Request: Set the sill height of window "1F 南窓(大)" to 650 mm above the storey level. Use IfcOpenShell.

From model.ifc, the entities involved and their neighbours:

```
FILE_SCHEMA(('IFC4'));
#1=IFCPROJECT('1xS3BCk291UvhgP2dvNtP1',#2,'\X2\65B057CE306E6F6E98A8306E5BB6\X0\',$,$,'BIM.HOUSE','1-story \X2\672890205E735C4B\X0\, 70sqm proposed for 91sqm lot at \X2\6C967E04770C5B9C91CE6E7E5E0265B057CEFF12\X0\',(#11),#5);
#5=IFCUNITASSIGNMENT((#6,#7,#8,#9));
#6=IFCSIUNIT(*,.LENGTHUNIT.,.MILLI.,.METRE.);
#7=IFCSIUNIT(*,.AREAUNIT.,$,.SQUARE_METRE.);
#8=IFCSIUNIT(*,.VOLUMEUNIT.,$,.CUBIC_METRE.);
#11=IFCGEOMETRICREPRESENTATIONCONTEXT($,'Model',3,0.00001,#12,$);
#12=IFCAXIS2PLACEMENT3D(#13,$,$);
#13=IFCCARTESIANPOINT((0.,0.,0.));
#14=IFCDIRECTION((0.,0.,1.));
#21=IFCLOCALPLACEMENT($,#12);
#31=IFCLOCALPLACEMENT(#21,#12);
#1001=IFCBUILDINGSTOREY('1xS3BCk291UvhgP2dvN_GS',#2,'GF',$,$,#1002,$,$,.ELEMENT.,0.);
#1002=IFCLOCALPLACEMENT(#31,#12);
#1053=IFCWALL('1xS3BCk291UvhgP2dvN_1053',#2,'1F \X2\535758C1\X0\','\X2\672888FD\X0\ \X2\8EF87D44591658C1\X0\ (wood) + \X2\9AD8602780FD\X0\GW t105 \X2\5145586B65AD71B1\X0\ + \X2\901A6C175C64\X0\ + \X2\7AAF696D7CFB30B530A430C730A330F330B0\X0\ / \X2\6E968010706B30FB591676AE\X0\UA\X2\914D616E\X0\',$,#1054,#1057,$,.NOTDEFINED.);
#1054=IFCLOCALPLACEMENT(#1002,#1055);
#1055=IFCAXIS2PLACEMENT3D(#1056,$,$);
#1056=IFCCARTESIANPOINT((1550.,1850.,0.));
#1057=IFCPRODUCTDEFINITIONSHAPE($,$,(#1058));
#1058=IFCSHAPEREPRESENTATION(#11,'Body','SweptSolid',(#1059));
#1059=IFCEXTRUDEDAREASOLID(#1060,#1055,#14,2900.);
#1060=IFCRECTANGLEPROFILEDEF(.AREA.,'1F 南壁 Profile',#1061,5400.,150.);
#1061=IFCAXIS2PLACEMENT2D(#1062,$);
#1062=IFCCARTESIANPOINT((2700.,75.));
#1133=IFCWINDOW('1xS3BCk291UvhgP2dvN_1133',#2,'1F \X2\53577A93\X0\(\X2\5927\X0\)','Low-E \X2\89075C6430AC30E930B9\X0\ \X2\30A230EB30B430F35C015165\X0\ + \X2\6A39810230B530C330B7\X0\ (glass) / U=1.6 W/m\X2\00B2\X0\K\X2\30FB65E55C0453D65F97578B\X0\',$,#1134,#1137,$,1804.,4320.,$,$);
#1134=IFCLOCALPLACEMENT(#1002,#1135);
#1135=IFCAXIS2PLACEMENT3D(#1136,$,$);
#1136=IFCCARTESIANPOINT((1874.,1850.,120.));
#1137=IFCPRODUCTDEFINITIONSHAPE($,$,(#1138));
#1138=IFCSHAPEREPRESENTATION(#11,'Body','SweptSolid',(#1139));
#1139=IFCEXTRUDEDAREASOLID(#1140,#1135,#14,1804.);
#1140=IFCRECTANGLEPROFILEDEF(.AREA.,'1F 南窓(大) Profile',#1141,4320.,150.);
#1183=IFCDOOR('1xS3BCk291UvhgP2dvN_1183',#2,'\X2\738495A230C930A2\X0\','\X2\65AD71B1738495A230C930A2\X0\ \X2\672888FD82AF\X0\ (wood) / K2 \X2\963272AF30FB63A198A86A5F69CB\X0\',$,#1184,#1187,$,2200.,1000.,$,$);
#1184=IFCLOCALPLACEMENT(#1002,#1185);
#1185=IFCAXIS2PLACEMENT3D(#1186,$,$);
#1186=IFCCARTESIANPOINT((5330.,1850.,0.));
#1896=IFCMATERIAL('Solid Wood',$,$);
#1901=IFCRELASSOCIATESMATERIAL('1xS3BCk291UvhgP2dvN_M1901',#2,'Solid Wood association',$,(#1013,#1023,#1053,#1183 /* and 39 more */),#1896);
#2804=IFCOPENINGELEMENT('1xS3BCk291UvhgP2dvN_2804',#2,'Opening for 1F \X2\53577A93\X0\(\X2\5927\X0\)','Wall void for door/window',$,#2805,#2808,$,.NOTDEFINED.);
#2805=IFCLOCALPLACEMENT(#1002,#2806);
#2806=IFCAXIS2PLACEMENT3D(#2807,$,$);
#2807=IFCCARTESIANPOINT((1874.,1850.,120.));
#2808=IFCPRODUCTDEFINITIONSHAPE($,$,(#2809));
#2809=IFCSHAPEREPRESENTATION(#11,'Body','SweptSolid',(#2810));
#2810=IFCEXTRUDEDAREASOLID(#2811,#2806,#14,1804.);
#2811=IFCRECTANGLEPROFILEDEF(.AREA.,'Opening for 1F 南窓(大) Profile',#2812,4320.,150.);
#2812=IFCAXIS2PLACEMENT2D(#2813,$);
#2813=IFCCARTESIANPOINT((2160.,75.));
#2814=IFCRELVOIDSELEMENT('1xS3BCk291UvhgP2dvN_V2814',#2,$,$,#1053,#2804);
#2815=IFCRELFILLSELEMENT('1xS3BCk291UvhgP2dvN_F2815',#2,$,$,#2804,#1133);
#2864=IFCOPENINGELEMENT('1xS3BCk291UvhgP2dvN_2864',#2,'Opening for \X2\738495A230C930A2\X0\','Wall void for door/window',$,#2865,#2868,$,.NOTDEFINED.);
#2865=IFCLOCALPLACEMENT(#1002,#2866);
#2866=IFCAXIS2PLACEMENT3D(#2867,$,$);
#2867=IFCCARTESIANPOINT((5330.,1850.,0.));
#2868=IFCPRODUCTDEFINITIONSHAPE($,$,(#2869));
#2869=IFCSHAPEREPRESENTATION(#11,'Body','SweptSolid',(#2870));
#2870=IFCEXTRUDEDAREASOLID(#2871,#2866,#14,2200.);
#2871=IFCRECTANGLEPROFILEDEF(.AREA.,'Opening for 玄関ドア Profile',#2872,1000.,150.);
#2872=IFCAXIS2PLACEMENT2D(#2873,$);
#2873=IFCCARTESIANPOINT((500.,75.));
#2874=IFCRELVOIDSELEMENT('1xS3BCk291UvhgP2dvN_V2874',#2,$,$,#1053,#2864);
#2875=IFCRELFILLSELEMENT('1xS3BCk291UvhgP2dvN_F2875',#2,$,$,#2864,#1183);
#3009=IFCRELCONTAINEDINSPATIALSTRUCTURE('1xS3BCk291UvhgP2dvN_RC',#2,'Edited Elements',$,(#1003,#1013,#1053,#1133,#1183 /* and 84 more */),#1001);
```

```python
import numpy as np
import ifcopenshell
import ifcopenshell.api.geometry
import ifcopenshell.geom
import ifcopenshell.util.element
import ifcopenshell.util.placement
import ifcopenshell.util.shape
import ifcopenshell.util.unit

model = ifcopenshell.open("model.ifc")
unit_scale = ifcopenshell.util.unit.calculate_unit_scale(model)

window = model.by_guid("1xS3BCk291UvhgP2dvN_1133")
opening = window.FillsVoids[0].RelatingOpeningElement
storey = ifcopenshell.util.element.get_container(window, ifc_class="IfcBuildingStorey")
level = ifcopenshell.util.placement.get_local_placement(storey.ObjectPlacement)[2, 3]

# The opening's origin need not be at the sill, so measure its lowest point.
shape = ifcopenshell.geom.create_shape(ifcopenshell.geom.settings(), opening)
bottom = ifcopenshell.util.shape.get_shape_bottom_elevation(shape, shape.geometry) / unit_scale
dz = level + 650.0 - bottom

shift = np.array([0.0, 0.0, dz])
# The window is not placed relative to its opening, so move both.
for product in (opening, window):
    matrix = ifcopenshell.util.placement.get_local_placement(product.ObjectPlacement)
    matrix[:3, 3] += shift
    ifcopenshell.api.geometry.edit_object_placement(model, product=product, matrix=matrix, is_si=False)

print(f"moved by {dz * unit_scale:+.3f} m")

model.write("model-out.ifc")
```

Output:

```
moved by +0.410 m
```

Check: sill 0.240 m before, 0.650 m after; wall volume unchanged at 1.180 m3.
